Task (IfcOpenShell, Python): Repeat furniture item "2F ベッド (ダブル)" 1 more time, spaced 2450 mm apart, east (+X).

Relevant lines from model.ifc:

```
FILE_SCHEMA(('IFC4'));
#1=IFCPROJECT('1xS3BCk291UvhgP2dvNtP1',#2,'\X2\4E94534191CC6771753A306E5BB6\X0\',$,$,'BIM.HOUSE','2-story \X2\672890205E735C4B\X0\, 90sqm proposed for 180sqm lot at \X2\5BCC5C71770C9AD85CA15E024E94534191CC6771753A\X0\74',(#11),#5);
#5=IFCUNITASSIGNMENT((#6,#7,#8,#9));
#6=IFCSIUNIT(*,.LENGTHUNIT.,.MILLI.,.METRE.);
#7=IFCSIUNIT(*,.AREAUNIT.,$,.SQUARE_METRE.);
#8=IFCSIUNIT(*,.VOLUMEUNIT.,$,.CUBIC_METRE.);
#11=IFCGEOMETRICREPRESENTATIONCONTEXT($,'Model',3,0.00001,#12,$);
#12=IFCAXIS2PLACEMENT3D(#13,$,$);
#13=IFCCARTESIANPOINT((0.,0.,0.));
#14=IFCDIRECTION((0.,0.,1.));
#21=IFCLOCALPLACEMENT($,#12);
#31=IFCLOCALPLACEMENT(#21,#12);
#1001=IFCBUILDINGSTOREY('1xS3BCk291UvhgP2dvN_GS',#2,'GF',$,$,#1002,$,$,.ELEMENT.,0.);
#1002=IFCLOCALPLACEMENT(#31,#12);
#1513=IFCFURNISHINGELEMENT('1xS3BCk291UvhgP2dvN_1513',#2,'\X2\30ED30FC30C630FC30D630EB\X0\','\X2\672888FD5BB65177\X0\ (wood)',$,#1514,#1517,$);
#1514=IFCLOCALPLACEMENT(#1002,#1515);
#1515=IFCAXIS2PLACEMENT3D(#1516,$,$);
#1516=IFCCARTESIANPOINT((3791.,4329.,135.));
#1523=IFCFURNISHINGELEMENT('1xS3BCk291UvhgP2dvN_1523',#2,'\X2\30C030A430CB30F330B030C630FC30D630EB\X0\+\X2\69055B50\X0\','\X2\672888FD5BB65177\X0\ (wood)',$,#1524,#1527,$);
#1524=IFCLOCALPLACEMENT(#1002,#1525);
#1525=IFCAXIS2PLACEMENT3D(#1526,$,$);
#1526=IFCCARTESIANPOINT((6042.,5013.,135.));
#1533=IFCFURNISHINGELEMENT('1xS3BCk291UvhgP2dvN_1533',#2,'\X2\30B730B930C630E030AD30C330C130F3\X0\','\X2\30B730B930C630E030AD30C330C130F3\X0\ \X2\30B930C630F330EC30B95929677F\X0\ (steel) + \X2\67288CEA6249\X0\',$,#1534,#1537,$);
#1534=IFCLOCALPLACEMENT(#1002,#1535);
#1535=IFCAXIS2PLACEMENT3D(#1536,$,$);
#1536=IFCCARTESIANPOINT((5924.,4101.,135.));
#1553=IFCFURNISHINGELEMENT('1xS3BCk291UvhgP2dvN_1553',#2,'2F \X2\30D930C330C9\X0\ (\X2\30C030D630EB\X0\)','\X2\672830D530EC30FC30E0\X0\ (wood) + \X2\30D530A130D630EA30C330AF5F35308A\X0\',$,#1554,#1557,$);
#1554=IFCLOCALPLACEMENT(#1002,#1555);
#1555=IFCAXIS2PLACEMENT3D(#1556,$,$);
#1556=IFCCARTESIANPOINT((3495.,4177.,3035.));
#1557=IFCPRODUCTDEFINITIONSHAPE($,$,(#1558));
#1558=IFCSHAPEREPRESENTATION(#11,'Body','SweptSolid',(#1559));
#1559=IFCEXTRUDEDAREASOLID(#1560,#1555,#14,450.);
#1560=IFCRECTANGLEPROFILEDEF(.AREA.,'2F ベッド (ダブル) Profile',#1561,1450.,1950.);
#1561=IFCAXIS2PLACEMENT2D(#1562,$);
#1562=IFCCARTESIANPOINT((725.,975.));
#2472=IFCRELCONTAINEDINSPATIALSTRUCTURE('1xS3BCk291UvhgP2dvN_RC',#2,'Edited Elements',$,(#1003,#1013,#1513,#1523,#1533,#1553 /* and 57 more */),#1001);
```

```python
import numpy as np
import ifcopenshell
import ifcopenshell.api.geometry
import ifcopenshell.api.root
import ifcopenshell.util.element
import ifcopenshell.util.placement

model = ifcopenshell.open("model.ifc")


def reuse_history(source, copy):
    """copy_class also copies each property set's owner history, people and application; keep the originals."""
    for rel in copy.IsDefinedBy:
        if rel.is_a("IfcRelDefinesByProperties") and (history := rel.RelatingPropertyDefinition.OwnerHistory):
            rel.RelatingPropertyDefinition.OwnerHistory = source.OwnerHistory
            ifcopenshell.util.element.remove_deep2(model, history)


source = model.by_guid("1xS3BCk291UvhgP2dvN_1553")
base = ifcopenshell.util.placement.get_local_placement(source.ObjectPlacement)
step = np.array([1.0, 0.0, 0.0]) * 2450.0

for i in range(1, 2):
    copy = ifcopenshell.api.root.copy_class(model, product=source)
    copy.Representation = ifcopenshell.util.element.copy_deep(
        model, source.Representation, exclude=["IfcGeometricRepresentationContext", "IfcRepresentationMap"]
    )
    reuse_history(source, copy)
    matrix = base.copy()
    matrix[:3, 3] += i * step
    print("added at", matrix[:3, 3].round(3) + 0.0)
    ifcopenshell.api.geometry.edit_object_placement(model, product=copy, matrix=matrix, is_si=False)

model.write("model-out.ifc")
```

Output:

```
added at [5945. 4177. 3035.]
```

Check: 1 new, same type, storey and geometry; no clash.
